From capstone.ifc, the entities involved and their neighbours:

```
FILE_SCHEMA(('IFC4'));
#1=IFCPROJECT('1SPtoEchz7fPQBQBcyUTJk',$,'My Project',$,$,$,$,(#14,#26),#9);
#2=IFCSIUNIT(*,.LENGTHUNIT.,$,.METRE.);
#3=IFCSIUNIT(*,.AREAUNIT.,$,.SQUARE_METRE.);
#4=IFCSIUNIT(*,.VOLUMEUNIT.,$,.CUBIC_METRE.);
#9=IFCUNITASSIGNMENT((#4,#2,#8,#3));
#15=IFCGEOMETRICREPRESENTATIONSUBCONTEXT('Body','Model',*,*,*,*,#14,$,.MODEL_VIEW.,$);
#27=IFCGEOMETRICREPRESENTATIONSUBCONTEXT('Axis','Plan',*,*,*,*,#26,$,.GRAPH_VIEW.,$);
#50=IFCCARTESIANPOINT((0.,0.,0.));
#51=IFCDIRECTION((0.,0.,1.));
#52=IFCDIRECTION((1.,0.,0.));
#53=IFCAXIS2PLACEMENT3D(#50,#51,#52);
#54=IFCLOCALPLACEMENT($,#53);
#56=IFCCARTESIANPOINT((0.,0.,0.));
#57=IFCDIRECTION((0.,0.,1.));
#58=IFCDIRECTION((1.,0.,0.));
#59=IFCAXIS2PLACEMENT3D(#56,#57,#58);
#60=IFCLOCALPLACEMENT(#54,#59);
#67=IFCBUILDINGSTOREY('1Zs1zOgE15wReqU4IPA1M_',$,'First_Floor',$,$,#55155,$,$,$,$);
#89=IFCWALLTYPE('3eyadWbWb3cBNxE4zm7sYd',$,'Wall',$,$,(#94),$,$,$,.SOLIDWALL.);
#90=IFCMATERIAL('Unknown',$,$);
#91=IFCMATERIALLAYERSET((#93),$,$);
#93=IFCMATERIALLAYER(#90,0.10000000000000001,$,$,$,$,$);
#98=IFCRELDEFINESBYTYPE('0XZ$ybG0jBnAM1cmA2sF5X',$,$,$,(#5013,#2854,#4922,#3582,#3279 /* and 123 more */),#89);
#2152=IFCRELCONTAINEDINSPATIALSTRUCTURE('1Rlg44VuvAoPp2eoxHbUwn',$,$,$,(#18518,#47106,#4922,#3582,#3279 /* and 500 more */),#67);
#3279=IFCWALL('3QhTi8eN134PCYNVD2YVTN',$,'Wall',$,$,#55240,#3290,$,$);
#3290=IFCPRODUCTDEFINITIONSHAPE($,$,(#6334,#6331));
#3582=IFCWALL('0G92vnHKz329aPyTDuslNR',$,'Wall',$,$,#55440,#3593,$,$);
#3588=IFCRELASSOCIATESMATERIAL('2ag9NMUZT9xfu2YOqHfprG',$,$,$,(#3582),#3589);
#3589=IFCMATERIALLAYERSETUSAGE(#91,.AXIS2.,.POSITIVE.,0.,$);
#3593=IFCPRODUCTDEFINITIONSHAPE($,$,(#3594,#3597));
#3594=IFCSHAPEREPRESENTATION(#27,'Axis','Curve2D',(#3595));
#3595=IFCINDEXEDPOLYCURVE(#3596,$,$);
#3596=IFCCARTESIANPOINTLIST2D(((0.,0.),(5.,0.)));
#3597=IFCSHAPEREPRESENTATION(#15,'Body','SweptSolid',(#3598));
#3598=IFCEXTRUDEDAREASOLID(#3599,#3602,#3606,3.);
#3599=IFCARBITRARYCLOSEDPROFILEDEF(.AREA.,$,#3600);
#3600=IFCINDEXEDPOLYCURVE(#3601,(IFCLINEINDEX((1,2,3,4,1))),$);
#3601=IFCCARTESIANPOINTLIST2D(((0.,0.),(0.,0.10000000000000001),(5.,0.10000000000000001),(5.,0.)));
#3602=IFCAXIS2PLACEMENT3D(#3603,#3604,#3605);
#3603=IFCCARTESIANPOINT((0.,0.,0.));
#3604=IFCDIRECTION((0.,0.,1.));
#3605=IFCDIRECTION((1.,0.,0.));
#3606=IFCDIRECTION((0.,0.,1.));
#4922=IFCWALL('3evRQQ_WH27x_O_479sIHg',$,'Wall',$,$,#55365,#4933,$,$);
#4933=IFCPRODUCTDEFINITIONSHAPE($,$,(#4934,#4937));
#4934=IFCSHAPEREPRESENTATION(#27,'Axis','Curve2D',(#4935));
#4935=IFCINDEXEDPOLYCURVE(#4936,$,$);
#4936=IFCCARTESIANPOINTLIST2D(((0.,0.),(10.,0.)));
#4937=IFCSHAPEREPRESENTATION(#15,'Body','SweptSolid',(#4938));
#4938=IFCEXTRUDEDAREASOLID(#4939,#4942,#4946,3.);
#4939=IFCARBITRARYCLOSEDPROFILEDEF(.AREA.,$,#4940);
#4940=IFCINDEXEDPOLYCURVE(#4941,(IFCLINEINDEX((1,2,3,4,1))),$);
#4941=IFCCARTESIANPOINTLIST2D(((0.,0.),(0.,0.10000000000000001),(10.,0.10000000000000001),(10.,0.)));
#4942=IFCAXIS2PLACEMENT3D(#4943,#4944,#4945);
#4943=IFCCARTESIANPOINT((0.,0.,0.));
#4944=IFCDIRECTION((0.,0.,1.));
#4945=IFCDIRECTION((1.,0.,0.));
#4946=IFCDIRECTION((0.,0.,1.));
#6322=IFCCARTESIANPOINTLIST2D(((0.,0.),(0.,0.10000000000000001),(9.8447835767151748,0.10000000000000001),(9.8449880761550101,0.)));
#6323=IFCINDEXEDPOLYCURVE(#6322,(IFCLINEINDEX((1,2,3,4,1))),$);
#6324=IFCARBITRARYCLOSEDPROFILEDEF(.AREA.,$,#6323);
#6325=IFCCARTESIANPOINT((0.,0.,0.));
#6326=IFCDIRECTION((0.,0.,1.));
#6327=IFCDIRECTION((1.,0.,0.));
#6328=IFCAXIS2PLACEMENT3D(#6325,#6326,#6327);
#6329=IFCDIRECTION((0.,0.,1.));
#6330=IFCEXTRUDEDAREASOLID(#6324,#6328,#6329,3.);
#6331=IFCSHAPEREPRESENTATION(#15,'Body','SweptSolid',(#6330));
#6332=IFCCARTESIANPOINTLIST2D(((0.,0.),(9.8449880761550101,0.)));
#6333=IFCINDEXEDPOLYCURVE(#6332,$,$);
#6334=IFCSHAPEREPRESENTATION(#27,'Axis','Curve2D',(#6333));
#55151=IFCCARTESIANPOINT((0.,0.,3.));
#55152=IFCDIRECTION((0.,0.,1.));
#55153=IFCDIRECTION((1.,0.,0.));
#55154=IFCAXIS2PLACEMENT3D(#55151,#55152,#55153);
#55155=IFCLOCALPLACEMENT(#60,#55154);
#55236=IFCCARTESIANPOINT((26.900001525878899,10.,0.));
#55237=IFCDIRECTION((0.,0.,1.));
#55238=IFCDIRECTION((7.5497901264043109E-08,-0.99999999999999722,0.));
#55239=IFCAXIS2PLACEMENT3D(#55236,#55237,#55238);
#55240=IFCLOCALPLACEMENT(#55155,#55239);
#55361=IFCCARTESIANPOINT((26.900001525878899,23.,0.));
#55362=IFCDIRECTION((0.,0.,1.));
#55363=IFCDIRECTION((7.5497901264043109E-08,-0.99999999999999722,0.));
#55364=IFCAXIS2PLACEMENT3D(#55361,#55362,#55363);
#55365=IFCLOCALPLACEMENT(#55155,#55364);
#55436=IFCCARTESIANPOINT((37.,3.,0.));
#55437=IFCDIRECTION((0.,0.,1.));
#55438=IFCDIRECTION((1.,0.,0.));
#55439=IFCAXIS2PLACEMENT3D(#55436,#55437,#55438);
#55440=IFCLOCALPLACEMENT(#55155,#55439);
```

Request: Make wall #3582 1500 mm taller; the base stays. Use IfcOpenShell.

```python
import ifcopenshell
import ifcopenshell.geom
import ifcopenshell.util.representation
import ifcopenshell.util.shape

model = ifcopenshell.open("capstone.ifc")
settings = ifcopenshell.geom.settings()


def volume(element):
    """Net volume in cubic metres, openings subtracted."""
    shape = ifcopenshell.geom.create_shape(settings, element)
    return ifcopenshell.util.shape.get_volume(shape.geometry)


wall = model.by_guid("0G92vnHKz329aPyTDuslNR")
before = volume(wall)

body = ifcopenshell.util.representation.get_representation(wall, "Model", "Body")
solid = body.Items[0]
old_height = solid.Depth
solid.Depth += 1.5
after = volume(wall)

print(f"height {old_height:g} -> {solid.Depth:g}, volume {before:.3f} -> {after:.3f} m3")

model.write("capstone_updated.ifc")
```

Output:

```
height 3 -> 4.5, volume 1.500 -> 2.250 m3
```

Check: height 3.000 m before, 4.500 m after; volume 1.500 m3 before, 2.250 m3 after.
